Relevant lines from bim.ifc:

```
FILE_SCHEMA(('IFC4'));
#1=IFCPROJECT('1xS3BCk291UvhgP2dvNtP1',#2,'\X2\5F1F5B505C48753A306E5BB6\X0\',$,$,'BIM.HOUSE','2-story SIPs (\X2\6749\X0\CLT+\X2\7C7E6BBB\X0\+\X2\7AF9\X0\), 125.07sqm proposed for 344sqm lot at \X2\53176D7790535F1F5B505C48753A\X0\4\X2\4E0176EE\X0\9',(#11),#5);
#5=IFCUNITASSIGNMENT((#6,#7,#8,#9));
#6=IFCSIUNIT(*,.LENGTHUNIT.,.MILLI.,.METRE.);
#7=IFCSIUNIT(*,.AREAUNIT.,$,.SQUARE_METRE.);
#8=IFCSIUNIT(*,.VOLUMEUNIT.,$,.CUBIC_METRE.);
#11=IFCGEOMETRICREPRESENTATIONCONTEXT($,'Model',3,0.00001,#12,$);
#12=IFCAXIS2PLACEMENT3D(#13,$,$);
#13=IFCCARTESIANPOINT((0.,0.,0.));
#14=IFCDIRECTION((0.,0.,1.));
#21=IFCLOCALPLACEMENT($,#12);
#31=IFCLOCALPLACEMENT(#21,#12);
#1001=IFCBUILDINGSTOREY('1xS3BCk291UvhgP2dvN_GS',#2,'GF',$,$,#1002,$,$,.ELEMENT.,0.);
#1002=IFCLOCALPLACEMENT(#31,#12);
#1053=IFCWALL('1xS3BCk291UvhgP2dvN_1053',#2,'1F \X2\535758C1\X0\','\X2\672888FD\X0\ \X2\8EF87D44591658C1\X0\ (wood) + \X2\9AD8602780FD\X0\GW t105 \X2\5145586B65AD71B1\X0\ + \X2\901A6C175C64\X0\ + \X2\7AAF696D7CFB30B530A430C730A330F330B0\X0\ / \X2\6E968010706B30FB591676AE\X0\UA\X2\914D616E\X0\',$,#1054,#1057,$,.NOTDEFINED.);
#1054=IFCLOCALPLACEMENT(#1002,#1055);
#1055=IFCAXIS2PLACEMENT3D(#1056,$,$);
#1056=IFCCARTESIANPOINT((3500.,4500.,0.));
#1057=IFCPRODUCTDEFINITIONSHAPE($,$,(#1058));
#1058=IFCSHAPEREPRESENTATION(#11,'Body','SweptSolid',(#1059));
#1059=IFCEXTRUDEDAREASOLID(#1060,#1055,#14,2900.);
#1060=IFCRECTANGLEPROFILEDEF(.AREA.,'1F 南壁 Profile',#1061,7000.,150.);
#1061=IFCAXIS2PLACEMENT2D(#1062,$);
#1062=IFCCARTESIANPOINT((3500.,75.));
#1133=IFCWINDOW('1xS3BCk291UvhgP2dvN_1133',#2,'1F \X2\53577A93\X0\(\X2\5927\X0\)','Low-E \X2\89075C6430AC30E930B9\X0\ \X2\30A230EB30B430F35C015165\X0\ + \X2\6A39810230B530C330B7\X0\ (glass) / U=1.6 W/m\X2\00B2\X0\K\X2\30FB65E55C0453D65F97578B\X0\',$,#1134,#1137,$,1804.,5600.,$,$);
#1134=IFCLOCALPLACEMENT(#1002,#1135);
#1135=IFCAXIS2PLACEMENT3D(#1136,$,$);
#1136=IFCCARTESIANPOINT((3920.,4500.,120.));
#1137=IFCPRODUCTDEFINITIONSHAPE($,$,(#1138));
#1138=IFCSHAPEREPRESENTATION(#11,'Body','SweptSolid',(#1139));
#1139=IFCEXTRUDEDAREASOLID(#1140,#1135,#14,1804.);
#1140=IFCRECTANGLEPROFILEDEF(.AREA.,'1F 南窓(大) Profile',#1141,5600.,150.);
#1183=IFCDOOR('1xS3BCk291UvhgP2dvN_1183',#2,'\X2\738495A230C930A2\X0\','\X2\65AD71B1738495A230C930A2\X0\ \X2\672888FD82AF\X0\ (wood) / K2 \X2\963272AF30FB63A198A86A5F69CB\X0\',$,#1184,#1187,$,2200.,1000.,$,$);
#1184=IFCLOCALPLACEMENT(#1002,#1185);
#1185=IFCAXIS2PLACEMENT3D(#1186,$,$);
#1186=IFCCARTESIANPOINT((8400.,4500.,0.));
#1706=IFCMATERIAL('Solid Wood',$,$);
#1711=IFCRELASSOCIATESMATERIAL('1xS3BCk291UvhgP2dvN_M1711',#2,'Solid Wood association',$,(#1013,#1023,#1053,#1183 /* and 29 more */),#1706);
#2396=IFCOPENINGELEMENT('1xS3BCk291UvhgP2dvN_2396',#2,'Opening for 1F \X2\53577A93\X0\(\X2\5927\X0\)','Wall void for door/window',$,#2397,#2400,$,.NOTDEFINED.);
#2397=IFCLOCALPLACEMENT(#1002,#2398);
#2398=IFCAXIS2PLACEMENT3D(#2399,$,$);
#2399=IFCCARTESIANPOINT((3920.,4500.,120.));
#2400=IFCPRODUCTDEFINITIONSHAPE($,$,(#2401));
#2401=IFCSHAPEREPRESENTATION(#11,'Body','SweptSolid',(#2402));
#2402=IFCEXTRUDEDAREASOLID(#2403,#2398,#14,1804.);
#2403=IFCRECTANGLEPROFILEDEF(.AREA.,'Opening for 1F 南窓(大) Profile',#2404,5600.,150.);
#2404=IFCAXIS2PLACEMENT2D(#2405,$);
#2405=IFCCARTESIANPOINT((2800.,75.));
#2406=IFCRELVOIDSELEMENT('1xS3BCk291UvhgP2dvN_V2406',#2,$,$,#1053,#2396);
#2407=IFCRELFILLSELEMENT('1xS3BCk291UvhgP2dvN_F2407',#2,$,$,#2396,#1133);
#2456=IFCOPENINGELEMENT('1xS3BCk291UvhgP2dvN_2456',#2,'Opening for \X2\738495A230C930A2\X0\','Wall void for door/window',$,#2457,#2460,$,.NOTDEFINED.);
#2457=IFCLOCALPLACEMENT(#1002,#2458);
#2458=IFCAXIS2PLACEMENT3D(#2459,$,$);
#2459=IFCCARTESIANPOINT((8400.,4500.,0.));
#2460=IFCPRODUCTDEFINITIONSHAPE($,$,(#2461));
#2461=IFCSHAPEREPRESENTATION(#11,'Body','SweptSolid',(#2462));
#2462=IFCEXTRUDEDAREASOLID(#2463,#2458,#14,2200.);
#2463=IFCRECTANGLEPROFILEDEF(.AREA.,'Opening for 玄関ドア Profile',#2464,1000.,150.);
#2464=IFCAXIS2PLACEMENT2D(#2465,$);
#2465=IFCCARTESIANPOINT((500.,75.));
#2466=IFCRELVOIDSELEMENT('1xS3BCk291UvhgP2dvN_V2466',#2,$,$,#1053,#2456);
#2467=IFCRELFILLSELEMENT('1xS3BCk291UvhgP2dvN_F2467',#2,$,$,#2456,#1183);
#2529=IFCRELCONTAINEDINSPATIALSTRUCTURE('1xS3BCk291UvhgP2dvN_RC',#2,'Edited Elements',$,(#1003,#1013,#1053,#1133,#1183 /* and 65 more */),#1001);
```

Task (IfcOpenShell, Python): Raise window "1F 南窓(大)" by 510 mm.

```python
import numpy as np
import ifcopenshell
import ifcopenshell.api.geometry
import ifcopenshell.util.placement
import ifcopenshell.util.unit

model = ifcopenshell.open("bim.ifc")
unit_scale = ifcopenshell.util.unit.calculate_unit_scale(model)

window = model.by_id(1133)
opening = window.FillsVoids[0].RelatingOpeningElement
dz = 0.51 / unit_scale

shift = np.array([0.0, 0.0, dz])
# The window is not placed relative to its opening, so move both.
for product in (opening, window):
    matrix = ifcopenshell.util.placement.get_local_placement(product.ObjectPlacement)
    matrix[:3, 3] += shift
    ifcopenshell.api.geometry.edit_object_placement(model, product=product, matrix=matrix, is_si=False)

print(f"moved by {dz * unit_scale:+.3f} m")

model.write("bim_rev.ifc")
```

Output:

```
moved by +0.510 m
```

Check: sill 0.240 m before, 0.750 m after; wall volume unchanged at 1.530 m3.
